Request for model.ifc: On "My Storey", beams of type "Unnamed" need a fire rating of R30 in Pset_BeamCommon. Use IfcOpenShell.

First a look at what the model holds.

```python
import ifcopenshell
import ifcopenshell.util.element

model = ifcopenshell.open("model.ifc")
print(model.schema)
storey = next(s for s in model.by_type("IfcBuildingStorey") if s.Name == "My Storey")
beams = [e for e in ifcopenshell.util.element.get_decomposition(storey) if e.is_a("IfcBeam")]
seen = {}
for e in beams:
    element_type = ifcopenshell.util.element.get_type(e)
    key = (element_type.Name if element_type != e and element_type else None, ifcopenshell.util.element.get_pset(e, "Pset_BeamCommon", "FireRating"))
    seen[key] = seen.get(key, 0) + 1
for (name, value), count in sorted(seen.items(), key=str):
    print(count, "x", name, "|", value)
```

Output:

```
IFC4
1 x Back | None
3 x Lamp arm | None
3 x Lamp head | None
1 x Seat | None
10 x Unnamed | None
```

```python
import ifcopenshell
import ifcopenshell.api.pset
import ifcopenshell.util.element

model = ifcopenshell.open("model.ifc")

storey = next(s for s in model.by_type("IfcBuildingStorey") if s.Name == "My Storey")
beams = [e for e in ifcopenshell.util.element.get_decomposition(storey) if e.is_a("IfcBeam")]

count = 0
for e in beams:
    element_type = ifcopenshell.util.element.get_type(e)
    if element_type in (None, e) or element_type.Name != "Unnamed":
        continue
    # add_pset returns the element's existing set when there is one.
    pset = ifcopenshell.api.pset.add_pset(model, product=e, name="Pset_BeamCommon")
    ifcopenshell.api.pset.edit_pset(model, pset=pset, properties={"FireRating": "R30"})
    count += 1

print(count, "beams updated")

model.write("model_updated.ifc")
```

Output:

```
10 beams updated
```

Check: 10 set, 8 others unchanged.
